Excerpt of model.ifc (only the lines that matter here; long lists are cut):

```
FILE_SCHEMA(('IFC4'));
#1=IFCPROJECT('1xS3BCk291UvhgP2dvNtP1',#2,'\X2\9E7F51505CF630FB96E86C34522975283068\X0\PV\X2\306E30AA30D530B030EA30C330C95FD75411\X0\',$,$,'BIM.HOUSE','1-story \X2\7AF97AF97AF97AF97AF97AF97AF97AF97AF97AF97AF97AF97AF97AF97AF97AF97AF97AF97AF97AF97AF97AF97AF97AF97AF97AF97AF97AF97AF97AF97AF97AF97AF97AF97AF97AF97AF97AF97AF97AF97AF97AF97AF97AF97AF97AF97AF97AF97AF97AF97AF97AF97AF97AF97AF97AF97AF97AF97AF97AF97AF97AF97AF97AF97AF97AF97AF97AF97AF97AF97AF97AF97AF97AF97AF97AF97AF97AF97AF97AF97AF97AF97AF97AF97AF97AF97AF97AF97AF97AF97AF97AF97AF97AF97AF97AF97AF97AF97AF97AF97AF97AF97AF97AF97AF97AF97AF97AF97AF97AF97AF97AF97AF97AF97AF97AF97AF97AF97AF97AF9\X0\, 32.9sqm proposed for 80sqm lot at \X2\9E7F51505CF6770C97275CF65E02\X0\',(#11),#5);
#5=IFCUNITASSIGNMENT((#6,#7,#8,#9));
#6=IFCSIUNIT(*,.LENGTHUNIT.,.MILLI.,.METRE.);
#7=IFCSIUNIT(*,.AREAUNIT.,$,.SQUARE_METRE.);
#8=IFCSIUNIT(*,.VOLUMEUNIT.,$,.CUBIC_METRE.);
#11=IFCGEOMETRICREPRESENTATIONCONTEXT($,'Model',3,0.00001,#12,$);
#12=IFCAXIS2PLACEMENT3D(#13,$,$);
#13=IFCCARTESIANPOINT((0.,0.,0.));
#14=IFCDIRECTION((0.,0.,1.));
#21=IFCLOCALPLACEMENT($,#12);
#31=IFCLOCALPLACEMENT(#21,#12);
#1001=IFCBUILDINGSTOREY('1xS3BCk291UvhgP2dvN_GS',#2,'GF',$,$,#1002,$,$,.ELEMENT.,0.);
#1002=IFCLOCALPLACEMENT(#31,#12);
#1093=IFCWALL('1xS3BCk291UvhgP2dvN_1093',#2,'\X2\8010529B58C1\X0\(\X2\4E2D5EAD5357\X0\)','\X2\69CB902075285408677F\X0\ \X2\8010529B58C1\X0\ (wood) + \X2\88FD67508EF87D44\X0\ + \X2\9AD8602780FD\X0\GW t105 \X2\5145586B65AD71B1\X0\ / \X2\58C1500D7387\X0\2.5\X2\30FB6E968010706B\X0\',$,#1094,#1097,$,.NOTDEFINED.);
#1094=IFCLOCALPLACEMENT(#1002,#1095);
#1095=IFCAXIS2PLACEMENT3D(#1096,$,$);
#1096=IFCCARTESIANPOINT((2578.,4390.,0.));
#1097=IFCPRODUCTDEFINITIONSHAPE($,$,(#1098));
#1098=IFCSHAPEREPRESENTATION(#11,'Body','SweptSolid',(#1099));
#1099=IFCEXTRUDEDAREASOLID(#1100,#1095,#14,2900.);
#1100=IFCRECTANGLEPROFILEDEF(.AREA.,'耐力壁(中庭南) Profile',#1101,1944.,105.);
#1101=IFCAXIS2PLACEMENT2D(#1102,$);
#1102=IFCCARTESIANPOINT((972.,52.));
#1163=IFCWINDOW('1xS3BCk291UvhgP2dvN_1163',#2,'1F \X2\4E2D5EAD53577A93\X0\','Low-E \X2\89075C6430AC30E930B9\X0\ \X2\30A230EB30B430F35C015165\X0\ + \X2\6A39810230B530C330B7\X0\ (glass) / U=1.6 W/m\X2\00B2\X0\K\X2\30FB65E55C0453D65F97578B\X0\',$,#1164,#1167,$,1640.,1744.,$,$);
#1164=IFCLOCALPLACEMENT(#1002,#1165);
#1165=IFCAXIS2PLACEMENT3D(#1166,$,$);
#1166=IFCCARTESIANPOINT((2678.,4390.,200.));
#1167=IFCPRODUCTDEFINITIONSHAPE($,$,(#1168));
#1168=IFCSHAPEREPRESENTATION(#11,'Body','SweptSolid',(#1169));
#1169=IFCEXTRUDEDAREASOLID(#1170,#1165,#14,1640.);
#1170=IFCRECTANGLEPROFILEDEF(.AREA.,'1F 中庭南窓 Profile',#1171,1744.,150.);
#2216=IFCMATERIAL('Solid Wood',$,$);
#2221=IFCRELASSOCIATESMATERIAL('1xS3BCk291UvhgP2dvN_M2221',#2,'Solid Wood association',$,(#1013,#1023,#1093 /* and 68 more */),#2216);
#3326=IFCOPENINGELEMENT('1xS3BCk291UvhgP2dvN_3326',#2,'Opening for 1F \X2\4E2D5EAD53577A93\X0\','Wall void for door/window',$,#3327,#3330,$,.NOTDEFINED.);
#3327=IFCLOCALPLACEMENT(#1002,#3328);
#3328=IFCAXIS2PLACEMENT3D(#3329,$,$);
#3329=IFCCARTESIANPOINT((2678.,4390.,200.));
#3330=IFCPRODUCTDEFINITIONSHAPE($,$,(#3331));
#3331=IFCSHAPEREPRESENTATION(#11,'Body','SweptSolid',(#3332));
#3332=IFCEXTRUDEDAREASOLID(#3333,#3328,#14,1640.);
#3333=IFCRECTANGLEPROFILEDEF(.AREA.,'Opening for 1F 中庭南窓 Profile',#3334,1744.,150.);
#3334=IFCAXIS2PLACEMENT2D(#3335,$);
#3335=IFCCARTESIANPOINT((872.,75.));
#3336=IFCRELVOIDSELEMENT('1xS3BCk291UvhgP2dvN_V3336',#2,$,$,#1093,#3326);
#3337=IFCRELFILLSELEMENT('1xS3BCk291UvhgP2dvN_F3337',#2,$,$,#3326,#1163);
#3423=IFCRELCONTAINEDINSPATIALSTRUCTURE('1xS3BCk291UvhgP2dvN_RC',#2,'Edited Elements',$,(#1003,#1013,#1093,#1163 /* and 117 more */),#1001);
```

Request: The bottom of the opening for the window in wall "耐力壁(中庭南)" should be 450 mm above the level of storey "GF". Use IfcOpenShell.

```python
import numpy as np
import ifcopenshell
import ifcopenshell.api.geometry
import ifcopenshell.geom
import ifcopenshell.util.element
import ifcopenshell.util.placement
import ifcopenshell.util.shape
import ifcopenshell.util.unit

model = ifcopenshell.open("model.ifc")
unit_scale = ifcopenshell.util.unit.calculate_unit_scale(model)

window = model.by_id(1163)
opening = window.FillsVoids[0].RelatingOpeningElement
storey = ifcopenshell.util.element.get_container(window, ifc_class="IfcBuildingStorey")
level = ifcopenshell.util.placement.get_local_placement(storey.ObjectPlacement)[2, 3]

# The opening's origin need not be at the sill, so measure its lowest point.
shape = ifcopenshell.geom.create_shape(ifcopenshell.geom.settings(), opening)
bottom = ifcopenshell.util.shape.get_shape_bottom_elevation(shape, shape.geometry) / unit_scale
dz = level + 0.45 / unit_scale - bottom

shift = np.array([0.0, 0.0, dz])
# The window is not placed relative to its opening, so move both.
for product in (opening, window):
    matrix = ifcopenshell.util.placement.get_local_placement(product.ObjectPlacement)
    matrix[:3, 3] += shift
    ifcopenshell.api.geometry.edit_object_placement(model, product=product, matrix=matrix, is_si=False)

print(f"moved by {dz * unit_scale:+.3f} m")

model.write("model_updated.ifc")
```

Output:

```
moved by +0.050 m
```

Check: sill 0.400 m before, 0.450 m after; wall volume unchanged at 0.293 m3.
